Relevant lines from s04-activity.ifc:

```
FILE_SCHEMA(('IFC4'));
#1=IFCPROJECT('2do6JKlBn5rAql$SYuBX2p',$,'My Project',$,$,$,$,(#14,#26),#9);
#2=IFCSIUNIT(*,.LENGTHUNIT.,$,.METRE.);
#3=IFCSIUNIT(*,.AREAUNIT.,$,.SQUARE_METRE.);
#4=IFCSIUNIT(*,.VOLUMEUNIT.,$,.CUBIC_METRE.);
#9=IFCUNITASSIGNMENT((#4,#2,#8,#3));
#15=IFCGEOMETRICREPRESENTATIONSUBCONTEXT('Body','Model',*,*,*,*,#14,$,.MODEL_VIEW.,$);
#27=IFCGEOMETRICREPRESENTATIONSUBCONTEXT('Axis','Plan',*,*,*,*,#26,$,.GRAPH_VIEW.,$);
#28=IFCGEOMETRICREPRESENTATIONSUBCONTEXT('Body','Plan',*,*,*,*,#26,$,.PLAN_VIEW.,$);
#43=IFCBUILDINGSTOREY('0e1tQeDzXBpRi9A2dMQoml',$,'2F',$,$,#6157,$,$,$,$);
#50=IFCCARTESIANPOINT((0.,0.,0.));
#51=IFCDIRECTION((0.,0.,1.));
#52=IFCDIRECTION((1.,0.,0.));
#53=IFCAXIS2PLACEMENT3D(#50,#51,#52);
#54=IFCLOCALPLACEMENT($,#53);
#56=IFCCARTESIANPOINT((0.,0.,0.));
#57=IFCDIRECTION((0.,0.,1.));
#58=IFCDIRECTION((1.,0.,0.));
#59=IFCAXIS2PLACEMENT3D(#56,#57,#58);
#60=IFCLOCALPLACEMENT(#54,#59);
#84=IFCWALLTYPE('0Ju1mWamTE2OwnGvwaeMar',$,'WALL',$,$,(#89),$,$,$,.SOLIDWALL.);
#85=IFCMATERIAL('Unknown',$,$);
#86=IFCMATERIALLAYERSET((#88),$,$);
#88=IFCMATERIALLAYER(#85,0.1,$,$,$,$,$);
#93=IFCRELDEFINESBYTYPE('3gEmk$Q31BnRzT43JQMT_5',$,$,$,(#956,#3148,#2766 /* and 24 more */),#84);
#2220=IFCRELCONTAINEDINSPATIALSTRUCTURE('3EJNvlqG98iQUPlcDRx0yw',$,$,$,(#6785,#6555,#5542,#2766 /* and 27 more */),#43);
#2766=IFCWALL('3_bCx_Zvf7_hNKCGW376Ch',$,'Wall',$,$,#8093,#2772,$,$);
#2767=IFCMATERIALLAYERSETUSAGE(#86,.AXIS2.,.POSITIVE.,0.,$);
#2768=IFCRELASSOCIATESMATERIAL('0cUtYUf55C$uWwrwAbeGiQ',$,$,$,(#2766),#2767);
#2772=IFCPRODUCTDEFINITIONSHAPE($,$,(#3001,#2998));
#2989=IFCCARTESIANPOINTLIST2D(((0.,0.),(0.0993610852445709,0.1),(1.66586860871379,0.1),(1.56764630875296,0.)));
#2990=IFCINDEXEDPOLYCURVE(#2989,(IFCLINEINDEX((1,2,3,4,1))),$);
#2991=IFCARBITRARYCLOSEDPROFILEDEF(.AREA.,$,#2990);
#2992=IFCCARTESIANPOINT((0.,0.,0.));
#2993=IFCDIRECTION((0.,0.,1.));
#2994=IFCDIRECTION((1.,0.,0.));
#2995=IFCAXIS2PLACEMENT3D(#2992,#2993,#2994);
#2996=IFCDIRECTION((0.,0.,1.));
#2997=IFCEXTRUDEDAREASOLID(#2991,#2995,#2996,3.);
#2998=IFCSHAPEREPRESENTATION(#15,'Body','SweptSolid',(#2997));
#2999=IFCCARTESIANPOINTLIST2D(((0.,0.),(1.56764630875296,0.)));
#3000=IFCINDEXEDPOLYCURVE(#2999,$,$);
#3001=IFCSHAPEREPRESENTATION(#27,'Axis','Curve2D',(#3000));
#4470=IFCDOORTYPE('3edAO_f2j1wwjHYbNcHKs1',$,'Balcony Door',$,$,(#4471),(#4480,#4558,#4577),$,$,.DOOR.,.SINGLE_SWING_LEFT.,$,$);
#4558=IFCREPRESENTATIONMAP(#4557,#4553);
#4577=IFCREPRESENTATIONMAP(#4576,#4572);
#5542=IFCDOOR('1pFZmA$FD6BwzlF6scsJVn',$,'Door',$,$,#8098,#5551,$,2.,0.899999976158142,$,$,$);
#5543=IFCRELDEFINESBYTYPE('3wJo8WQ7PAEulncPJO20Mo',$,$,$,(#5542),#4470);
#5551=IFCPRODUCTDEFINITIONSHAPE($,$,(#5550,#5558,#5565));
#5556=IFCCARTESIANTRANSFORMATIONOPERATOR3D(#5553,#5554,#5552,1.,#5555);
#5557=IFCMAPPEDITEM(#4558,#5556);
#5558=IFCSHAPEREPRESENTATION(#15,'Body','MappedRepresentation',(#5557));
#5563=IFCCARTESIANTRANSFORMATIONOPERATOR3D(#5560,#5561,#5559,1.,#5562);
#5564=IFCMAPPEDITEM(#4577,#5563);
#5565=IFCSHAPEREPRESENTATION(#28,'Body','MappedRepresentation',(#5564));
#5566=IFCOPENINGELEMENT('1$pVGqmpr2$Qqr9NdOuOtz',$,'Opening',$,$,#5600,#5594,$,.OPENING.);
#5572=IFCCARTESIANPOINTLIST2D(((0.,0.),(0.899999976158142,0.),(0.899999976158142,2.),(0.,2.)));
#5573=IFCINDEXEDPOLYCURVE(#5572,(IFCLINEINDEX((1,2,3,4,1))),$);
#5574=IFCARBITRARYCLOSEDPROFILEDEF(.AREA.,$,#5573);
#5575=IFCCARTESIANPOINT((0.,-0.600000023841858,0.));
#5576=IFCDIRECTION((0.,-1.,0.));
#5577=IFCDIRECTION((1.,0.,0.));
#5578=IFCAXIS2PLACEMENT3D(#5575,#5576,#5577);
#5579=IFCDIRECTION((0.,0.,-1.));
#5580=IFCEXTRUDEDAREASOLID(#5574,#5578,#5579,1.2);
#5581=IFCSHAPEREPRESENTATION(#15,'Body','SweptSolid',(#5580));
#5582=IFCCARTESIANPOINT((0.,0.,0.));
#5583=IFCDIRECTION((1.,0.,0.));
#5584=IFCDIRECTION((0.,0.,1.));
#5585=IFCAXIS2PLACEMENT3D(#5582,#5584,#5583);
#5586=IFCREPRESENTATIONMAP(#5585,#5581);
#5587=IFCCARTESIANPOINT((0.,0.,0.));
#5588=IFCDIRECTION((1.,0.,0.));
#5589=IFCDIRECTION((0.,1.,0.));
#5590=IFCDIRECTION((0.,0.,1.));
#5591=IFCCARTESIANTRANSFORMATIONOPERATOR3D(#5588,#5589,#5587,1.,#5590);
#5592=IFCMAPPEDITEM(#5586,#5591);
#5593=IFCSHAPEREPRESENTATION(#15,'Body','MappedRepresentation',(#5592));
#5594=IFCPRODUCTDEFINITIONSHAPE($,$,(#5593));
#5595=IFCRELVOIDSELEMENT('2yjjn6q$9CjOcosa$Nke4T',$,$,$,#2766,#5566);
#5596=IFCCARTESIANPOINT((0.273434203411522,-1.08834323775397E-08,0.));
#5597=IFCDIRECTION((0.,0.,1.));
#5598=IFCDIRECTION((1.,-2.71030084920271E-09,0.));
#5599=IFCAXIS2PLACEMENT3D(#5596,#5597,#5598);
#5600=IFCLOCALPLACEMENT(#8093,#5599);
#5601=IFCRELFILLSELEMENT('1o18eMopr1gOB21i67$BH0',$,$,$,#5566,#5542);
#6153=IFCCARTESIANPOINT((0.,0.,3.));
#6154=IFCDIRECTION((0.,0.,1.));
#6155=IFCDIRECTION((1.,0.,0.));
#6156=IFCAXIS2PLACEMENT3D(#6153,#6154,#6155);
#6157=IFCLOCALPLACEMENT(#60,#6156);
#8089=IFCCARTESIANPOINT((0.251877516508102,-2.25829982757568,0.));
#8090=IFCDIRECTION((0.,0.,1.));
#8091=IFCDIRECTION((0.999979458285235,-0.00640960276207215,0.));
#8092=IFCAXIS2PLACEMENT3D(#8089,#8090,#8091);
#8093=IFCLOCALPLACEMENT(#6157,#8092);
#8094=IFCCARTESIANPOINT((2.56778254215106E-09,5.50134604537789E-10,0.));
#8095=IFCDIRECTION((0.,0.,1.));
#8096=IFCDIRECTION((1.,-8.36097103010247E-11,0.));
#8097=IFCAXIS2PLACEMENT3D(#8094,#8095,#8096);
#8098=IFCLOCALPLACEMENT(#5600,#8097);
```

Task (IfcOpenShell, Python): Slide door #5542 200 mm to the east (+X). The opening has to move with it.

```python
import ifcopenshell
import ifcopenshell.api.geometry
import ifcopenshell.util.placement
import ifcopenshell.util.unit

model = ifcopenshell.open("s04-activity.ifc")
unit_scale = ifcopenshell.util.unit.calculate_unit_scale(model)

door = model.by_guid("1pFZmA$FD6BwzlF6scsJVn")
opening = door.FillsVoids[0].RelatingOpeningElement
wall = opening.VoidsElements[0].RelatingBuildingElement

wall_matrix = ifcopenshell.util.placement.get_local_placement(wall.ObjectPlacement)
shift = wall_matrix[:3, 0] * 0.2 / unit_scale
before = ifcopenshell.util.placement.get_local_placement(door.ObjectPlacement)[:3, 3].copy()

# The door is placed relative to its opening, so it follows when the opening moves.
matrix = ifcopenshell.util.placement.get_local_placement(opening.ObjectPlacement)
matrix[:3, 3] += shift
ifcopenshell.api.geometry.edit_object_placement(
    model, product=opening, matrix=matrix, is_si=False, should_transform_children=True
)

after = ifcopenshell.util.placement.get_local_placement(door.ObjectPlacement)[:3, 3]
print("door moved by", (after - before).round(3) + 0.0)

model.write("s04-activity_rev.ifc")
```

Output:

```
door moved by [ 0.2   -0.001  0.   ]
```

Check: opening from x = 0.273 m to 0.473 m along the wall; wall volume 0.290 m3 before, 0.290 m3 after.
